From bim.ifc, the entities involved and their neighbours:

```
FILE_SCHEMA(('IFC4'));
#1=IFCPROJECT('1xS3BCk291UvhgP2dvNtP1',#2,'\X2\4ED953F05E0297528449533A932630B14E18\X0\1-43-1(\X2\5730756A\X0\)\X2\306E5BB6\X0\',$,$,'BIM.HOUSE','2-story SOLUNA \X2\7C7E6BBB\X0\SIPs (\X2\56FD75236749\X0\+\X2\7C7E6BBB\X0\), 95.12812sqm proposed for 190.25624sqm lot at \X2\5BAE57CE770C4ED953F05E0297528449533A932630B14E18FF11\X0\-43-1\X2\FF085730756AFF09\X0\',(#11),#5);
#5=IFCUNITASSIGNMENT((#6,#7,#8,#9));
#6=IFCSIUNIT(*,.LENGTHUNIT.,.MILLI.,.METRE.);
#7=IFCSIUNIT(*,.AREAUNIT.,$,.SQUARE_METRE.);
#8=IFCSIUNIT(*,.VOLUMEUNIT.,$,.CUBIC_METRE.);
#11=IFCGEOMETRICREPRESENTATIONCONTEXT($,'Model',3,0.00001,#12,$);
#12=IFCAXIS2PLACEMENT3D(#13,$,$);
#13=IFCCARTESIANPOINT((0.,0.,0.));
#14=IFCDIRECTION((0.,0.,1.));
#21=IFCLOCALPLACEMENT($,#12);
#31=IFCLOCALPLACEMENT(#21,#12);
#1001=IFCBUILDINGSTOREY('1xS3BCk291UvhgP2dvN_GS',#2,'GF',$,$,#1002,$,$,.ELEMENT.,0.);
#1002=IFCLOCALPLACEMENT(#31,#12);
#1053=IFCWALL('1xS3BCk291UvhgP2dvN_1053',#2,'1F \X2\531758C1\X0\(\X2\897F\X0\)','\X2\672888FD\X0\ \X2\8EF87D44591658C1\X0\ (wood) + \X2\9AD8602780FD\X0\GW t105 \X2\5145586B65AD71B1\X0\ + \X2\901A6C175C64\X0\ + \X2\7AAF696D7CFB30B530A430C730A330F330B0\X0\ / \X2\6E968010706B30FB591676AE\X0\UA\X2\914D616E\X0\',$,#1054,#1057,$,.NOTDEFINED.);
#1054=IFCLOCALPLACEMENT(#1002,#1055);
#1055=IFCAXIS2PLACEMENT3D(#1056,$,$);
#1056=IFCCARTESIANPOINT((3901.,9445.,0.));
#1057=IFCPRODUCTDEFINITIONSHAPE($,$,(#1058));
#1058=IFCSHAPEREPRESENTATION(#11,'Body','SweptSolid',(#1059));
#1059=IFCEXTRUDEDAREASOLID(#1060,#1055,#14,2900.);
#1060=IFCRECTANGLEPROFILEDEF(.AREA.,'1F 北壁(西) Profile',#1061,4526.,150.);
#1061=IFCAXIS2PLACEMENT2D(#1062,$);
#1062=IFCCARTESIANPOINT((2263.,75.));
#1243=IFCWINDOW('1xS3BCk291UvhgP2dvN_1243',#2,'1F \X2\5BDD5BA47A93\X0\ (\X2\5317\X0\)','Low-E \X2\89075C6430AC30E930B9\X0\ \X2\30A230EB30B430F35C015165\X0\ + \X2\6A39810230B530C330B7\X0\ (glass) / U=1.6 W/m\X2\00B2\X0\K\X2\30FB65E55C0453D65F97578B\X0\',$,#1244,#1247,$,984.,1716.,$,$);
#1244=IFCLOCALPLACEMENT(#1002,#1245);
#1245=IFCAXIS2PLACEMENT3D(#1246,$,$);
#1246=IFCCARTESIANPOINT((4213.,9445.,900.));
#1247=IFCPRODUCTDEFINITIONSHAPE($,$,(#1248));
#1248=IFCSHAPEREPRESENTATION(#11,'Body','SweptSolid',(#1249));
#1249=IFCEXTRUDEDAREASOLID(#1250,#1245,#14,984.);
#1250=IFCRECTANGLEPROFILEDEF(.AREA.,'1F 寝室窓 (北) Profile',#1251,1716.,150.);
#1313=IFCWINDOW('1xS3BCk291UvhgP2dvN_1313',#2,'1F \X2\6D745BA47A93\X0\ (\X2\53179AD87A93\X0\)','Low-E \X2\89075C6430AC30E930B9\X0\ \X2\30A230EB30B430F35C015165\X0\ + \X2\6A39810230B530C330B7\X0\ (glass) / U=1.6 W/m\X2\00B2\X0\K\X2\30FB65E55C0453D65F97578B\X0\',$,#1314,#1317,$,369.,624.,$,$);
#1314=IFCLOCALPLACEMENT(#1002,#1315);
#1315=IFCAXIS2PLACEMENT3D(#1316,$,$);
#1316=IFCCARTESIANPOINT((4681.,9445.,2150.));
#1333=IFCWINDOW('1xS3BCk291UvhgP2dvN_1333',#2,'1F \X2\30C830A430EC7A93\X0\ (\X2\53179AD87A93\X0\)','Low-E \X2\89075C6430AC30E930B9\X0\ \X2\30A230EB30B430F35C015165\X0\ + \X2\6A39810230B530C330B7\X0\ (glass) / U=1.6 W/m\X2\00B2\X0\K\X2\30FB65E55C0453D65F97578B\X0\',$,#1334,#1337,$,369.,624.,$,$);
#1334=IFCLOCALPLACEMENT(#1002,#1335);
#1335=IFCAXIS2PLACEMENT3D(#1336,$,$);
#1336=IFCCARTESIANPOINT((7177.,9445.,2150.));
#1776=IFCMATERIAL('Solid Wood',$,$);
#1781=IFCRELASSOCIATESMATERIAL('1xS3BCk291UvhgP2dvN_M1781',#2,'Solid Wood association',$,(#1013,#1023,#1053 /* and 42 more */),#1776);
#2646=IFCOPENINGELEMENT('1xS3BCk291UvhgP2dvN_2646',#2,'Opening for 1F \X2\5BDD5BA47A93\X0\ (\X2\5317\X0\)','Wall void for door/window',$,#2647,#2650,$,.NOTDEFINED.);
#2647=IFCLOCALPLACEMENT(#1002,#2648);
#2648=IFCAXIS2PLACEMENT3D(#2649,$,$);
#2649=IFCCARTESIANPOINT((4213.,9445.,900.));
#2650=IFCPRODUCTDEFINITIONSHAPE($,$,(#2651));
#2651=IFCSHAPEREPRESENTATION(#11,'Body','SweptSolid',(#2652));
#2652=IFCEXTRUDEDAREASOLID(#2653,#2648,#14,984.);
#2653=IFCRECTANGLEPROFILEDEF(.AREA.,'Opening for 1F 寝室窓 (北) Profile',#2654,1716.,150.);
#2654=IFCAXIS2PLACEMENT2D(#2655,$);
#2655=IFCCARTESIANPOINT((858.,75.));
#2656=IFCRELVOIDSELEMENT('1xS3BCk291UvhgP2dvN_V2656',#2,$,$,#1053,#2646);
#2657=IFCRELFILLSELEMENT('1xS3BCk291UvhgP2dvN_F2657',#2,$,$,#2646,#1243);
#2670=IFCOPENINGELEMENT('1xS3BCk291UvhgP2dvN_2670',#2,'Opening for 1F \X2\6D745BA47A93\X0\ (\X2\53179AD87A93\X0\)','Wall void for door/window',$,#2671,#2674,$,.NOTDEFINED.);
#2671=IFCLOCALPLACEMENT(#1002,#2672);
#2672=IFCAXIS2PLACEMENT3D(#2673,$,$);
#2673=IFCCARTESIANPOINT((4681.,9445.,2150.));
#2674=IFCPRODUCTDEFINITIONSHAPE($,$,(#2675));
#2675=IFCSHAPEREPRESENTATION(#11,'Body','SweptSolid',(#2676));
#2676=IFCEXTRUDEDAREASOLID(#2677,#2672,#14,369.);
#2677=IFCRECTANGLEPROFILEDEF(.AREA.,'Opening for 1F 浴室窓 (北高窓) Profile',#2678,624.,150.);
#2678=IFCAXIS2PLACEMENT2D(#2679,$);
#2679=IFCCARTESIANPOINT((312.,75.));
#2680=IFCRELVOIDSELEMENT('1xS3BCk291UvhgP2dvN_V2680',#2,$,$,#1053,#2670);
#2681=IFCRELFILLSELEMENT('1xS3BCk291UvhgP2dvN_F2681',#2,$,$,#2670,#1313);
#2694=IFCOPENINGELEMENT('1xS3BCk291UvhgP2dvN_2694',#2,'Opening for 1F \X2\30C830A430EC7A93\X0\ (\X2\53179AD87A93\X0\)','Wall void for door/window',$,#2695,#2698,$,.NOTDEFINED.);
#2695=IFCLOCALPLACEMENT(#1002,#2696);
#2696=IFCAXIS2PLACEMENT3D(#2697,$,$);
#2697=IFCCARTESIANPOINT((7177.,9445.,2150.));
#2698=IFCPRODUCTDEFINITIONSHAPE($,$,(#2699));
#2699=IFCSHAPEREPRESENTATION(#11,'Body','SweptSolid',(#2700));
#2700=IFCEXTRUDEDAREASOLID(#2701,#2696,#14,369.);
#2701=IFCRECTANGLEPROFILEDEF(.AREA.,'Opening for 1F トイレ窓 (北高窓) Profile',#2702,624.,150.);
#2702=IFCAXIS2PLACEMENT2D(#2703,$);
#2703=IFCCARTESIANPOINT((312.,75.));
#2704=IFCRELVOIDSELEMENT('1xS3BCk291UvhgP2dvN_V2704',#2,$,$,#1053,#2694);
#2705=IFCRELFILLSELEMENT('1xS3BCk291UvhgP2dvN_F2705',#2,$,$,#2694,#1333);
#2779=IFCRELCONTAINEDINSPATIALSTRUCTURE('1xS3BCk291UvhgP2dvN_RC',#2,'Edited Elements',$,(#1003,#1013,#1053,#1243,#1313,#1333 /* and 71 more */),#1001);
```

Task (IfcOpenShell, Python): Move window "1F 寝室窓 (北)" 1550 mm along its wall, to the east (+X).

```python
import ifcopenshell
import ifcopenshell.api.geometry
import ifcopenshell.util.placement
import ifcopenshell.util.unit

model = ifcopenshell.open("bim.ifc")
unit_scale = ifcopenshell.util.unit.calculate_unit_scale(model)

window = model.by_guid("1xS3BCk291UvhgP2dvN_1243")
opening = window.FillsVoids[0].RelatingOpeningElement
wall = opening.VoidsElements[0].RelatingBuildingElement

wall_matrix = ifcopenshell.util.placement.get_local_placement(wall.ObjectPlacement)
shift = wall_matrix[:3, 0] * 1.55 / unit_scale
before = ifcopenshell.util.placement.get_local_placement(window.ObjectPlacement)[:3, 3].copy()

# The window is not placed relative to its opening, so move both.
for product in (opening, window):
    matrix = ifcopenshell.util.placement.get_local_placement(product.ObjectPlacement)
    matrix[:3, 3] += shift
    ifcopenshell.api.geometry.edit_object_placement(model, product=product, matrix=matrix, is_si=False)

after = ifcopenshell.util.placement.get_local_placement(window.ObjectPlacement)[:3, 3]
print("window moved by", (after - before).round(3) + 0.0)

model.write("bim_rev.ifc")
```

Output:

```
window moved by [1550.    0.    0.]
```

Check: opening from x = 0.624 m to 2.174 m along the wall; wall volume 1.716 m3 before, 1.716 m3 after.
